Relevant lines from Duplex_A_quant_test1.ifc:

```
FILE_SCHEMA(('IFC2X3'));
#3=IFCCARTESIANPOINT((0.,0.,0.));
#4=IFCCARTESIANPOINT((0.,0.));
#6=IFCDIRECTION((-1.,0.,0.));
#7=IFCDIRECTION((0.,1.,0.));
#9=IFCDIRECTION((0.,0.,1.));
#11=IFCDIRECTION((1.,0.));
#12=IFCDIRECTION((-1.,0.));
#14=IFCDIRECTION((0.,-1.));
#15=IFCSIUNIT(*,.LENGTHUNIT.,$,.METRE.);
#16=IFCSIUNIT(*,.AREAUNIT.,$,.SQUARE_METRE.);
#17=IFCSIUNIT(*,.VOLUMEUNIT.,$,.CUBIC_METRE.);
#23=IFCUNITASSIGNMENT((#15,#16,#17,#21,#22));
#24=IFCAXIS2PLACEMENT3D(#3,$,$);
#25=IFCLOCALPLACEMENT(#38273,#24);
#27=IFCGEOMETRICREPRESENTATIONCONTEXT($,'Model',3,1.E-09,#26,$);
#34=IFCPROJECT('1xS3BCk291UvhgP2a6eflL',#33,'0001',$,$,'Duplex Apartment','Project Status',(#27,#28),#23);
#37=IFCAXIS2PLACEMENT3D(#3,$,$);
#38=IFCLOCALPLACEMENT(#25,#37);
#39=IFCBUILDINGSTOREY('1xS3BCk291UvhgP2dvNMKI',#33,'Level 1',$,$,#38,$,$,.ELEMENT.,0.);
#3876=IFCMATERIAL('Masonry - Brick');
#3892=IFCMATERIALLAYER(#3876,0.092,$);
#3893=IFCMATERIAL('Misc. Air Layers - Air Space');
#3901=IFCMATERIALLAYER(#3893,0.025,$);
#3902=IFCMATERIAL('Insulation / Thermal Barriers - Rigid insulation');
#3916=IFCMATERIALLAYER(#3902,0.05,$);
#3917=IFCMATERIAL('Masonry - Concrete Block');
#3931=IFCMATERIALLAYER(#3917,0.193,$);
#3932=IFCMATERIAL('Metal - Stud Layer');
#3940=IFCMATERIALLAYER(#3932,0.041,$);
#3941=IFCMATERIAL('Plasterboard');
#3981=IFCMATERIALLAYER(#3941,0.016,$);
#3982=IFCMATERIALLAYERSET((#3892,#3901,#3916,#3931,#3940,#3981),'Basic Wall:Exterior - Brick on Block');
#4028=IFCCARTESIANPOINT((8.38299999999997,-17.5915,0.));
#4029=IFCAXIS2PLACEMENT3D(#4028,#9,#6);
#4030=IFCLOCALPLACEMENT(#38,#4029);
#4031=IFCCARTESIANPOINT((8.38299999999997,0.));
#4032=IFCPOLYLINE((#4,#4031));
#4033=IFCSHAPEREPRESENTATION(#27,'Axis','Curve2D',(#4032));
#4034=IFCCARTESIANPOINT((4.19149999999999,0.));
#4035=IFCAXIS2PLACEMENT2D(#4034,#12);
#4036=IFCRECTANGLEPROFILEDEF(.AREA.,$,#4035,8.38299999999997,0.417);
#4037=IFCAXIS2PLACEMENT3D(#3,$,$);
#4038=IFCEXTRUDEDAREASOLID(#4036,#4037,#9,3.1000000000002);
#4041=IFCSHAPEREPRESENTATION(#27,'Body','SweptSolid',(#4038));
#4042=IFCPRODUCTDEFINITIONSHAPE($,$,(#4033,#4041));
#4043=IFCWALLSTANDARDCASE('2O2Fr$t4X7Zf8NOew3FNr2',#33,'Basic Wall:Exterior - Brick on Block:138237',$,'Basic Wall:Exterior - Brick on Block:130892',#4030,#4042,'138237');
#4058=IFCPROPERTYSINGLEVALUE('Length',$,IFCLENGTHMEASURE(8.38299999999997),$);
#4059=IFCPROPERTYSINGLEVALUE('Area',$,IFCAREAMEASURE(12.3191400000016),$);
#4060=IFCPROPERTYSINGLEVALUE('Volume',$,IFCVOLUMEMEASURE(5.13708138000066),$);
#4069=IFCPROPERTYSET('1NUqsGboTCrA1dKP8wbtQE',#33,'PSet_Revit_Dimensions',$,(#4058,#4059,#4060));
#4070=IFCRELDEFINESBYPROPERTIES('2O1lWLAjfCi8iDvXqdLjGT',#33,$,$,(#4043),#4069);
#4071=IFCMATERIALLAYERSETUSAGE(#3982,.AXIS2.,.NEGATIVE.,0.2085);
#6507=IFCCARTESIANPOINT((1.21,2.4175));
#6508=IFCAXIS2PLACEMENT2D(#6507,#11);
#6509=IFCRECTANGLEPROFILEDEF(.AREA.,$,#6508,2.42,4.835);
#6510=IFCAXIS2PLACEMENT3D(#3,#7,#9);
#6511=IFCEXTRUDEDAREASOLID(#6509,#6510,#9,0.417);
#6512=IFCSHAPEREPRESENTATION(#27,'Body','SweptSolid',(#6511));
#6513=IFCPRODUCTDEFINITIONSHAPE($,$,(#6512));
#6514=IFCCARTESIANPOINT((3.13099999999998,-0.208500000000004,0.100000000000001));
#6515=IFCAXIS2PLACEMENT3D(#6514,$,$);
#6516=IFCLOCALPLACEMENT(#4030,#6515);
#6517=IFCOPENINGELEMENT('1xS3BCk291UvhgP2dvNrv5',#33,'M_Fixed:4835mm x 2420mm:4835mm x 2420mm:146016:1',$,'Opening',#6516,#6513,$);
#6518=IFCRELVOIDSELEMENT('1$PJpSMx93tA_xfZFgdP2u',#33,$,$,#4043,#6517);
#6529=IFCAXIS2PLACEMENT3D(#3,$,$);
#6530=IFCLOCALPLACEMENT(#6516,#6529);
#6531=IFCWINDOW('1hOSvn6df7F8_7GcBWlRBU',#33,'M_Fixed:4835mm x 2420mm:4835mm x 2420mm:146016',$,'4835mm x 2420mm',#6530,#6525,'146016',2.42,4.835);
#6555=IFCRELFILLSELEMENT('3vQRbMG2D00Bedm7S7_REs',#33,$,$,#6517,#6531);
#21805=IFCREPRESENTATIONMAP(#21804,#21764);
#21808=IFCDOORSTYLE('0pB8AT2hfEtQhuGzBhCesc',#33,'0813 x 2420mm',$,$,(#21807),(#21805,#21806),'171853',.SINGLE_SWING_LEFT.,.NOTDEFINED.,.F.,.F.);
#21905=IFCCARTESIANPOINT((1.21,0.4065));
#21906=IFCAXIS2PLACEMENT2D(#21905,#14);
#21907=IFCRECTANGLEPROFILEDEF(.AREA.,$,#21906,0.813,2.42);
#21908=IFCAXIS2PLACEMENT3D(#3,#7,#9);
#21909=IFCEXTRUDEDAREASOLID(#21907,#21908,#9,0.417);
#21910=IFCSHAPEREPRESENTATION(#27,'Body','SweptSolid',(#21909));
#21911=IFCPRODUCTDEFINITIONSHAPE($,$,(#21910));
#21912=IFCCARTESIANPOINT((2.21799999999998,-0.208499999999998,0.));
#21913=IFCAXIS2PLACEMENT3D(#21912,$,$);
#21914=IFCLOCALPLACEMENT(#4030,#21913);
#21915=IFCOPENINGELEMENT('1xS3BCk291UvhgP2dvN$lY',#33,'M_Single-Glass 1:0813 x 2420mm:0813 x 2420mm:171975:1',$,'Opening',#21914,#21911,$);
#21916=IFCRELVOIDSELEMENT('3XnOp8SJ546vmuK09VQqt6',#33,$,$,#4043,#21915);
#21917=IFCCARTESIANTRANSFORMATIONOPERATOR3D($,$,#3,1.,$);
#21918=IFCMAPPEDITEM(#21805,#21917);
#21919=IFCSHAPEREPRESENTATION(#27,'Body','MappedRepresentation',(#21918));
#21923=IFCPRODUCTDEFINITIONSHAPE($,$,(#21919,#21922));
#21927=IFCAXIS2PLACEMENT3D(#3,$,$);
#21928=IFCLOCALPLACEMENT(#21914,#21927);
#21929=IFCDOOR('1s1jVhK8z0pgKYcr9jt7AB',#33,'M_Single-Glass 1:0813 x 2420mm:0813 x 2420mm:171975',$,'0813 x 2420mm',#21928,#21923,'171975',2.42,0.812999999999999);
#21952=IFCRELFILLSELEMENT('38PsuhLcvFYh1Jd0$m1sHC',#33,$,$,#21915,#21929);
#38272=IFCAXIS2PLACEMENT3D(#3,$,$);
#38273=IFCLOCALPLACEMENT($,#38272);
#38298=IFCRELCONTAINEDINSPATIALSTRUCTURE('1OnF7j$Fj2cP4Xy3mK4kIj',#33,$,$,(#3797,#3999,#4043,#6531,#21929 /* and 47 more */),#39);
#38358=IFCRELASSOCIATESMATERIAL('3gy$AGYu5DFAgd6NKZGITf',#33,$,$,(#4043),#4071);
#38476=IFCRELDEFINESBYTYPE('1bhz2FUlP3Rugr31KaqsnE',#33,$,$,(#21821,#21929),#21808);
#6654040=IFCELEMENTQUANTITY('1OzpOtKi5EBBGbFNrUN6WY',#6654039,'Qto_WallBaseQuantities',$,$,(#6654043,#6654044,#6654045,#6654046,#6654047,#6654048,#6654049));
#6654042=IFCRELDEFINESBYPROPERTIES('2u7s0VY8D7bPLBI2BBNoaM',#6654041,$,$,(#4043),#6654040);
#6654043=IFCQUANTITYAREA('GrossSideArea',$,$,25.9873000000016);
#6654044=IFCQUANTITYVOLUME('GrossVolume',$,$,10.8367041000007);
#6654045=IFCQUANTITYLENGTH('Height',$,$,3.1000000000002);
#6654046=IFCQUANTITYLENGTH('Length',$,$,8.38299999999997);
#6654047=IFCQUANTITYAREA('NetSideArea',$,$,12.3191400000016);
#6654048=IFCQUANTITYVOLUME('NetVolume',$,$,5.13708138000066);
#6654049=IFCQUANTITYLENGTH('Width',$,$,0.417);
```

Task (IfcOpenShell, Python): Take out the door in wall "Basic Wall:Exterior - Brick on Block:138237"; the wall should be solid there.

```python
import ifcopenshell
import ifcopenshell.api.feature
import ifcopenshell.api.pset
import ifcopenshell.api.root
import ifcopenshell.geom
import ifcopenshell.util.element
import ifcopenshell.util.shape
import ifcopenshell.util.unit

model = ifcopenshell.open("Duplex_A_quant_test1.ifc")
area_scale = ifcopenshell.util.unit.calculate_unit_scale(model, "AREAUNIT")
volume_scale = ifcopenshell.util.unit.calculate_unit_scale(model, "VOLUMEUNIT")
settings = ifcopenshell.geom.settings()


def volume(element):
    """Net volume in cubic metres, openings subtracted."""
    shape = ifcopenshell.geom.create_shape(settings, element)
    return ifcopenshell.util.shape.get_volume(shape.geometry)


door = model.by_guid("1s1jVhK8z0pgKYcr9jt7AB")
opening = door.FillsVoids[0].RelatingOpeningElement
wall = opening.VoidsElements[0].RelatingBuildingElement
before = volume(wall)

ifcopenshell.api.root.remove_product(model, product=door)
ifcopenshell.api.feature.remove_feature(model, feature=opening)

after = volume(wall)
thickness = 0.417  # wall thickness in metres

# Update the wall's stored quantities.
pset = model.by_id(ifcopenshell.util.element.get_pset(wall, "PSet_Revit_Dimensions", should_inherit=False)["id"])
ifcopenshell.api.pset.edit_pset(model, pset=pset, properties={
    "Area": model.create_entity("IfcAreaMeasure", after / thickness / area_scale),
    "Volume": model.create_entity("IfcVolumeMeasure", after / volume_scale),
})
qto = model.by_id(ifcopenshell.util.element.get_pset(wall, "Qto_WallBaseQuantities", should_inherit=False)["id"])
ifcopenshell.api.pset.edit_qto(model, qto=qto, properties={
    "NetSideArea": after / thickness / area_scale,
    "NetVolume": after / volume_scale,
})

print(f"wall volume {before:.3f} -> {after:.3f} m3")

model.write("Duplex_A_quant_test1_updated.ifc")
```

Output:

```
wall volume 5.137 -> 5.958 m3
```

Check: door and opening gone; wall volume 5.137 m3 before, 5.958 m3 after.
